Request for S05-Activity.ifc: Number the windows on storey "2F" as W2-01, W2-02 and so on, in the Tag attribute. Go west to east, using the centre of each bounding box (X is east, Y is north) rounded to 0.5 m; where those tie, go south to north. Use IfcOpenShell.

First a look at what the model holds.

```python
import ifcopenshell
import ifcopenshell.util.element
import ifcopenshell.util.placement

model = ifcopenshell.open("S05-Activity.ifc")
print(model.schema)
storey = next(s for s in model.by_type("IfcBuildingStorey") if s.Name == "2F")
windows = [e for e in ifcopenshell.util.element.get_decomposition(storey) if e.is_a("IfcWindow")]
for e in sorted(windows, key=lambda e: e.id()):
    origin = ifcopenshell.util.placement.get_local_placement(e.ObjectPlacement)[:3, 3]
    print(e.id(), e.Tag, e.Name, origin.round(2) + 0.0, sep=" | ")
```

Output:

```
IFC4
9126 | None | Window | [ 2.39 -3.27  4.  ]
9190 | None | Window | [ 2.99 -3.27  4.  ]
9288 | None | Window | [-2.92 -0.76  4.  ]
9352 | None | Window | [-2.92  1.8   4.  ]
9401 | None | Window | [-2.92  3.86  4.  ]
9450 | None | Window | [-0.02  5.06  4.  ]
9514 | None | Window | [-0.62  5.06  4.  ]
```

```python
import ifcopenshell
import ifcopenshell.geom
import ifcopenshell.util.element
import ifcopenshell.util.shape

model = ifcopenshell.open("S05-Activity.ifc")
settings = ifcopenshell.geom.settings()
settings.set("use-world-coords", True)


def centre(element):
    shape = ifcopenshell.geom.create_shape(settings, element)
    return ifcopenshell.util.shape.get_bbox_centroid(shape.geometry)


storey = next(s for s in model.by_type("IfcBuildingStorey") if s.Name == "2F")
windows = [e for e in ifcopenshell.util.element.get_decomposition(storey) if e.is_a("IfcWindow")]

# Insertion points can sit at a corner or the storey origin, so sort by the geometry (in metres).
centres = {e: centre(e) for e in windows}
windows.sort(key=lambda e: (round(centres[e][0] / 0.5), centres[e][1]))

for i, e in enumerate(windows, start=1):
    number = f"W2-{i:02d}"
    e.Tag = number
    print(e.id(), number)

model.write("S05-Activity_updated.ifc")
```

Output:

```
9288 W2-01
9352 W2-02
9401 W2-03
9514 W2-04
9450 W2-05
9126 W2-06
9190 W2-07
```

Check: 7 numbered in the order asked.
